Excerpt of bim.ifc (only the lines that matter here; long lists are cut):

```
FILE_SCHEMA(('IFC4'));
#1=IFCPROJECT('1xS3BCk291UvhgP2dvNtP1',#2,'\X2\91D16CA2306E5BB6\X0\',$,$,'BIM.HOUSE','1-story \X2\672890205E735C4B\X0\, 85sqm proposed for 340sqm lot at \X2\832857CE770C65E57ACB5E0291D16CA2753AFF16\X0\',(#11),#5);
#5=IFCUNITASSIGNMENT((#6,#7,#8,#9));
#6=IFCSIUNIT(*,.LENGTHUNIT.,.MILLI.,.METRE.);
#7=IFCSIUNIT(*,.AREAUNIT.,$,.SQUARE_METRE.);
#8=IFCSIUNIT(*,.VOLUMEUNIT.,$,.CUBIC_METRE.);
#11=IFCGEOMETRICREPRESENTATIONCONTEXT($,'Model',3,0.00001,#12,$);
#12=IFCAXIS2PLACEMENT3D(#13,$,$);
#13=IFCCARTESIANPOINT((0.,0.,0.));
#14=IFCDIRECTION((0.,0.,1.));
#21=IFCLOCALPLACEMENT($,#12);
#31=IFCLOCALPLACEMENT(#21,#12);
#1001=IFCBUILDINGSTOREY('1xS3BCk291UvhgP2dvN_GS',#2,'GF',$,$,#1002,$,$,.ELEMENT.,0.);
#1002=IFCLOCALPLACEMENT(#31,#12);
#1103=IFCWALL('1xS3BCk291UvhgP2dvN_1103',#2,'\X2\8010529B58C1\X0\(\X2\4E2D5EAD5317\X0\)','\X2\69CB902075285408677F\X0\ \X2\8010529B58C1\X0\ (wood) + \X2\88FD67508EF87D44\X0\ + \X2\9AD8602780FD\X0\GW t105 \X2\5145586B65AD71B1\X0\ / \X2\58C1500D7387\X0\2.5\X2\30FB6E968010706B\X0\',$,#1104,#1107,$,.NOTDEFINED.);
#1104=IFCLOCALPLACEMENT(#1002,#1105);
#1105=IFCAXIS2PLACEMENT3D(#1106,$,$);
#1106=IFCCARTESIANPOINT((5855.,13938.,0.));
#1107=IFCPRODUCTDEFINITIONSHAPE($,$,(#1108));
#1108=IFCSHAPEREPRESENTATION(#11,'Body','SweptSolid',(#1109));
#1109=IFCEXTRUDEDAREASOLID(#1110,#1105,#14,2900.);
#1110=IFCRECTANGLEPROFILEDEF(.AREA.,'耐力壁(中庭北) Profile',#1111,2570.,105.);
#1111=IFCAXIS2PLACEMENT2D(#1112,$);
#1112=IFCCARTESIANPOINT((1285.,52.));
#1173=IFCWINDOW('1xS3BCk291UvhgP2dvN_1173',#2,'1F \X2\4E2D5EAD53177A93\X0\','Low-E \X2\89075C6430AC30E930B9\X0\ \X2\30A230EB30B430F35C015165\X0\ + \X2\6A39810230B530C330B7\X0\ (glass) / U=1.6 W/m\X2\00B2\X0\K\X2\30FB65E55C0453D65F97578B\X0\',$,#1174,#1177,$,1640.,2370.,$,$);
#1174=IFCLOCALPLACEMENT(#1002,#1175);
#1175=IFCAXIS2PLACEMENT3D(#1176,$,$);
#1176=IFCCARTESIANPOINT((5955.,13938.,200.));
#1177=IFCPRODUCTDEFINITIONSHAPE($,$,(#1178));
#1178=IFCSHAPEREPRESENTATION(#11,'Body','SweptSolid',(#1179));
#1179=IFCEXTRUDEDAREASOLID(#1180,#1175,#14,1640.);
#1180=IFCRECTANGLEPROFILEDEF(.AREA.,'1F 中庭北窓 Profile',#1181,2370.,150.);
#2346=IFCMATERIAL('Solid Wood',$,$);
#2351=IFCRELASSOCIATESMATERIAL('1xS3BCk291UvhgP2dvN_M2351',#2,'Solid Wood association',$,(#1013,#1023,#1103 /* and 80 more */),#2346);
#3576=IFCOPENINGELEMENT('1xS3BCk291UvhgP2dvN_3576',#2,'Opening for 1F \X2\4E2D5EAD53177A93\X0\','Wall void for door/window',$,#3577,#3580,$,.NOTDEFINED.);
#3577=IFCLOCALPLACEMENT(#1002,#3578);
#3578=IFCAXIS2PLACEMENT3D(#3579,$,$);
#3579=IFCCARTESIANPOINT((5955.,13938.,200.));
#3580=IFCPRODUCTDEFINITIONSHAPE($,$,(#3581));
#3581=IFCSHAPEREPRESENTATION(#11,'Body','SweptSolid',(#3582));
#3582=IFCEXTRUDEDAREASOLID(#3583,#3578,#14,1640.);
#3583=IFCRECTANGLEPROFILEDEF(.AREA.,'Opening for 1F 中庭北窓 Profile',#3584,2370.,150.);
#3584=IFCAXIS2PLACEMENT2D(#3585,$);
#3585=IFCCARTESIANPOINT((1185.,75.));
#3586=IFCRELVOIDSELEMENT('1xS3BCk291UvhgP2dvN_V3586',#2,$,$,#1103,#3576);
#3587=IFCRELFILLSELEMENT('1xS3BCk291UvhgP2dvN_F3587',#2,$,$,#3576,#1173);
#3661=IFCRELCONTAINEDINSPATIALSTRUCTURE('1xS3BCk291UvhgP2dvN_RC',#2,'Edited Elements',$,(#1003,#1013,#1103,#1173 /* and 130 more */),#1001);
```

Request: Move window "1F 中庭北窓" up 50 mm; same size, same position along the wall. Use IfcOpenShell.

```python
import numpy as np
import ifcopenshell
import ifcopenshell.api.geometry
import ifcopenshell.util.placement
import ifcopenshell.util.unit

model = ifcopenshell.open("bim.ifc")
unit_scale = ifcopenshell.util.unit.calculate_unit_scale(model)

window = model.by_guid("1xS3BCk291UvhgP2dvN_1173")
opening = window.FillsVoids[0].RelatingOpeningElement
dz = 50.0

shift = np.array([0.0, 0.0, dz])
# The window is not placed relative to its opening, so move both.
for product in (opening, window):
    matrix = ifcopenshell.util.placement.get_local_placement(product.ObjectPlacement)
    matrix[:3, 3] += shift
    ifcopenshell.api.geometry.edit_object_placement(model, product=product, matrix=matrix, is_si=False)

print(f"moved by {dz * unit_scale:+.3f} m")

model.write("bim_edited.ifc")
```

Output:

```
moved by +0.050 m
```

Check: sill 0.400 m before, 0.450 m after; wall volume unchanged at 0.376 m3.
